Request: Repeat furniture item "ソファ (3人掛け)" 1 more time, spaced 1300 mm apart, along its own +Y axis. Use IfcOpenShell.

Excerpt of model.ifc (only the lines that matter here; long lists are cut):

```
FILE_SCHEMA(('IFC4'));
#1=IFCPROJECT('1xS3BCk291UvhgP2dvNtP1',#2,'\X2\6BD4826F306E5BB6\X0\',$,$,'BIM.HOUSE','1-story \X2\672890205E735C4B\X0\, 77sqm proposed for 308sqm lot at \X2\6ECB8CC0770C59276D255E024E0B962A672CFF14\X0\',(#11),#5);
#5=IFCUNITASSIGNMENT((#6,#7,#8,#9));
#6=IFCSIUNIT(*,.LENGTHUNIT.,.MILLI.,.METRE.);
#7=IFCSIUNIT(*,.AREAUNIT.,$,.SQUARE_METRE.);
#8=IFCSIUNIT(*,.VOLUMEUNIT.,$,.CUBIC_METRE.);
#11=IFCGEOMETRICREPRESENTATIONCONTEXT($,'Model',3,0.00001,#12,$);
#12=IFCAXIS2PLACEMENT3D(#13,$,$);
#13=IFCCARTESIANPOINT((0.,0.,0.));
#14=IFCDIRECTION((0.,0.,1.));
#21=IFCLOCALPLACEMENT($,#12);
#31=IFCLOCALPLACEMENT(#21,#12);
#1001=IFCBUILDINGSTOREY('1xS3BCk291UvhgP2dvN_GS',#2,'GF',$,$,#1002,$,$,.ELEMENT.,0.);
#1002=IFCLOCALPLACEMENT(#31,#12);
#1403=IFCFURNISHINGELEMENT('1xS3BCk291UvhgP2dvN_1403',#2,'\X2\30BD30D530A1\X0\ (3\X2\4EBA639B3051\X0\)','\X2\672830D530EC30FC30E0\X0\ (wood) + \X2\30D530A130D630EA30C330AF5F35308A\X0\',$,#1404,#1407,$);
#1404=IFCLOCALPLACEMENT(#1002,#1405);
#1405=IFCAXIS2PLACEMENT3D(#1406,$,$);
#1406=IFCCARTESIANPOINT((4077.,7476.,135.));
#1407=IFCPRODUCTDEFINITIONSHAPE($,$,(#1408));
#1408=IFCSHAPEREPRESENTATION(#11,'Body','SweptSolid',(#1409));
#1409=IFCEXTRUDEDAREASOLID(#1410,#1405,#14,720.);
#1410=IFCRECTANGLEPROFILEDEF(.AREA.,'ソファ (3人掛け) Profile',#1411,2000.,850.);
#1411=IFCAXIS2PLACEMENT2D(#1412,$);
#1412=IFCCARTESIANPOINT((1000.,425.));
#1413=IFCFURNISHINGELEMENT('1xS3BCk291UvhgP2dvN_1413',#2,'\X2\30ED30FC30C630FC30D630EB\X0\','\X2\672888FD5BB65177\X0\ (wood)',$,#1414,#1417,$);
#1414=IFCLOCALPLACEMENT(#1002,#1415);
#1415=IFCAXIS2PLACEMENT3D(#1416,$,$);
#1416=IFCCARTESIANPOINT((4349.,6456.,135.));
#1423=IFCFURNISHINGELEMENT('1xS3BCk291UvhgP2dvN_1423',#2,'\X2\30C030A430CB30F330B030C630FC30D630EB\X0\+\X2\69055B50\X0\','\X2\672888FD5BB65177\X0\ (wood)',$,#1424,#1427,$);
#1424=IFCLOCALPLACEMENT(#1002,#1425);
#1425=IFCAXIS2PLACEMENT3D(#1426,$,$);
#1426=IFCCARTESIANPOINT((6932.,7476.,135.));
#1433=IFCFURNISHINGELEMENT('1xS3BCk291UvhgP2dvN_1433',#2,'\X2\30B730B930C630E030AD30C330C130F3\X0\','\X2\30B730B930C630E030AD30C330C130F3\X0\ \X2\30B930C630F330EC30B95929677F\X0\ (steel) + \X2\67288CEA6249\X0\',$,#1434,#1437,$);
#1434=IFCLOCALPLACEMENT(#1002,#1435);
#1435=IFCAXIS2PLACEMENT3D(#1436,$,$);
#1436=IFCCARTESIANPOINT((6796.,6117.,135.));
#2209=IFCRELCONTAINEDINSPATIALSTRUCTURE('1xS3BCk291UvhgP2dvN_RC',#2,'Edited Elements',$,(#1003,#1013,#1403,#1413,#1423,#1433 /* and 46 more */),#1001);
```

```python
import ifcopenshell
import ifcopenshell.api.geometry
import ifcopenshell.api.root
import ifcopenshell.util.element
import ifcopenshell.util.placement

model = ifcopenshell.open("model.ifc")


def reuse_history(source, copy):
    """copy_class also copies each property set's owner history, people and application; keep the originals."""
    for rel in copy.IsDefinedBy:
        if rel.is_a("IfcRelDefinesByProperties") and (history := rel.RelatingPropertyDefinition.OwnerHistory):
            rel.RelatingPropertyDefinition.OwnerHistory = source.OwnerHistory
            ifcopenshell.util.element.remove_deep2(model, history)


source = model.by_id(1403)
base = ifcopenshell.util.placement.get_local_placement(source.ObjectPlacement)
step = base[:3, 1] * 1300.0

for i in range(1, 2):
    copy = ifcopenshell.api.root.copy_class(model, product=source)
    copy.Representation = ifcopenshell.util.element.copy_deep(
        model, source.Representation, exclude=["IfcGeometricRepresentationContext", "IfcRepresentationMap"]
    )
    reuse_history(source, copy)
    matrix = base.copy()
    matrix[:3, 3] += i * step
    print("added at", matrix[:3, 3].round(3) + 0.0)
    ifcopenshell.api.geometry.edit_object_placement(model, product=copy, matrix=matrix, is_si=False)

model.write("model_edited.ifc")
```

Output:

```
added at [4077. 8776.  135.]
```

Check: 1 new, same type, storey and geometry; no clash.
